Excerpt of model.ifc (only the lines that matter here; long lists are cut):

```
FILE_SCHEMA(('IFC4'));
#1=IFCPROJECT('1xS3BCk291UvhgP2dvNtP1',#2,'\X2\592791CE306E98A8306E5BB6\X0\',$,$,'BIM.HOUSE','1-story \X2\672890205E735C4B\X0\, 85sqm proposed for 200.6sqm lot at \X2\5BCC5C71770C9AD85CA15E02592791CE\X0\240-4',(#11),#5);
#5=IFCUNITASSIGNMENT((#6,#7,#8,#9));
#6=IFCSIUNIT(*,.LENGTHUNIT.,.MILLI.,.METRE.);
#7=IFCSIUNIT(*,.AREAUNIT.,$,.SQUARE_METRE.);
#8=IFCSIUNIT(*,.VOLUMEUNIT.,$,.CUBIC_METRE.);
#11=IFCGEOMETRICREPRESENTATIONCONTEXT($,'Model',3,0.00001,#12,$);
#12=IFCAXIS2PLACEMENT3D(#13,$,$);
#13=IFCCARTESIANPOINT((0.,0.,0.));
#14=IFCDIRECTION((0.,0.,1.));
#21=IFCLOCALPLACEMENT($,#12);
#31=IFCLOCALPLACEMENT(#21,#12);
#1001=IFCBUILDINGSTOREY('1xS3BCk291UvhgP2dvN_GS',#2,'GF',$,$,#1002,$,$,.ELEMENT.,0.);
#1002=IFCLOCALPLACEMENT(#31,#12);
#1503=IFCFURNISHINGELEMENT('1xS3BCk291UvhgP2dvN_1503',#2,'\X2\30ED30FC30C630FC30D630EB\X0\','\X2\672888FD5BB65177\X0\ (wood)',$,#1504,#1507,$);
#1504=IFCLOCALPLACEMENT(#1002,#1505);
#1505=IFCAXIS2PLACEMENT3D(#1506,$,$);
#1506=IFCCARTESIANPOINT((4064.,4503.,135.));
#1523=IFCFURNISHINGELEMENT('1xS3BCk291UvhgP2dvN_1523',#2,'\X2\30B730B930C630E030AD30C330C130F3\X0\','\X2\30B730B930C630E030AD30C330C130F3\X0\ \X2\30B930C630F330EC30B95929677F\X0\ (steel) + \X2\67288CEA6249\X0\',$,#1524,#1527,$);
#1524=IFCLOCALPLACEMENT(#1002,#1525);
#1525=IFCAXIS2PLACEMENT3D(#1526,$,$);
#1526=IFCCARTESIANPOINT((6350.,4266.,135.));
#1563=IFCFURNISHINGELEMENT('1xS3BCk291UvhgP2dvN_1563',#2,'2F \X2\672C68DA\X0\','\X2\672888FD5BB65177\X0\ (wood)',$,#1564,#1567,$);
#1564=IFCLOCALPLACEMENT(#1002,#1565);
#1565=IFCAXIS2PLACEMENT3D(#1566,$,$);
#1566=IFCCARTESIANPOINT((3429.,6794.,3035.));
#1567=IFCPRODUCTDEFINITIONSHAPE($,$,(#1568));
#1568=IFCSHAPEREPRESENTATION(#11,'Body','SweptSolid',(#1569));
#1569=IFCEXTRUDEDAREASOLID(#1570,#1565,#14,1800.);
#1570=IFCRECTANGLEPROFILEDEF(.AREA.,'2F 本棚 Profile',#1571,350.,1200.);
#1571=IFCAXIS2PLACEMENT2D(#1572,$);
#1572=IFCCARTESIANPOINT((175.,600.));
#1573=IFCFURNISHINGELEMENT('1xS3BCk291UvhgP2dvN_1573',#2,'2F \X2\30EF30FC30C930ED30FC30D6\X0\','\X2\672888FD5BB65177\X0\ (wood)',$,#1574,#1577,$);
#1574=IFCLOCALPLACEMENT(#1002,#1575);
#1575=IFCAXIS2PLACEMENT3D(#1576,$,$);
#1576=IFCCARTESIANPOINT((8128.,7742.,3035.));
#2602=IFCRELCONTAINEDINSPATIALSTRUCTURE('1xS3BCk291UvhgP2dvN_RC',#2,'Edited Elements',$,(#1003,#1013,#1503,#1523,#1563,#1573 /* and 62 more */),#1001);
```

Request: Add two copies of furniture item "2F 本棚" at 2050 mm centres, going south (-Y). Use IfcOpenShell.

```python
import numpy as np
import ifcopenshell
import ifcopenshell.api.geometry
import ifcopenshell.api.root
import ifcopenshell.util.element
import ifcopenshell.util.placement
import ifcopenshell.util.unit

model = ifcopenshell.open("model.ifc")
unit_scale = ifcopenshell.util.unit.calculate_unit_scale(model)


def reuse_history(source, copy):
    """copy_class also copies each property set's owner history, people and application; keep the originals."""
    for rel in copy.IsDefinedBy:
        if rel.is_a("IfcRelDefinesByProperties") and (history := rel.RelatingPropertyDefinition.OwnerHistory):
            rel.RelatingPropertyDefinition.OwnerHistory = source.OwnerHistory
            ifcopenshell.util.element.remove_deep2(model, history)


source = model.by_guid("1xS3BCk291UvhgP2dvN_1563")
base = ifcopenshell.util.placement.get_local_placement(source.ObjectPlacement)
step = np.array([0.0, -1.0, 0.0]) * 2.05 / unit_scale

for i in range(1, 3):
    copy = ifcopenshell.api.root.copy_class(model, product=source)
    copy.Representation = ifcopenshell.util.element.copy_deep(
        model, source.Representation, exclude=["IfcGeometricRepresentationContext", "IfcRepresentationMap"]
    )
    reuse_history(source, copy)
    matrix = base.copy()
    matrix[:3, 3] += i * step
    print("added at", matrix[:3, 3].round(3) + 0.0)
    ifcopenshell.api.geometry.edit_object_placement(model, product=copy, matrix=matrix, is_si=False)

model.write("model_edited.ifc")
```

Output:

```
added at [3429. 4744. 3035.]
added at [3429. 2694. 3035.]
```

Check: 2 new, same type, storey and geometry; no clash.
